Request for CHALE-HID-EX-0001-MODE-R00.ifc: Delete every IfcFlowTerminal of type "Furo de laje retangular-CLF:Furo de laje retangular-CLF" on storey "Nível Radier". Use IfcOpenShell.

First a look at what the model holds.

```python
import ifcopenshell
import ifcopenshell.util.element

model = ifcopenshell.open("CHALE-HID-EX-0001-MODE-R00.ifc")
print(model.schema)
storey = next(s for s in model.by_type("IfcBuildingStorey") if s.Name == "Nível Radier")
terminals = [e for e in ifcopenshell.util.element.get_decomposition(storey) if e.is_a("IfcFlowTerminal")]
seen = {}
for e in terminals:
    element_type = ifcopenshell.util.element.get_type(e)
    name = element_type.Name if element_type not in (None, e) else None
    seen[name] = seen.get(name, 0) + 1
for name, count in sorted(seen.items(), key=str):
    print(count, "x", name)
```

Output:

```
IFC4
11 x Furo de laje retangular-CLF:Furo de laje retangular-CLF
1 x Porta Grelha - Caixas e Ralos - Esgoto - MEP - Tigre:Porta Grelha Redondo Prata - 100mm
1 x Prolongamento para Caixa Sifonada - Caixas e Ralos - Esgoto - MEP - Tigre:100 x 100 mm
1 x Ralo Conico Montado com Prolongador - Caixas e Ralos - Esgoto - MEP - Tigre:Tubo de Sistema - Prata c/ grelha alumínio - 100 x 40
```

```python
import ifcopenshell
import ifcopenshell.api.root
import ifcopenshell.util.element

model = ifcopenshell.open("CHALE-HID-EX-0001-MODE-R00.ifc")

storey = next(s for s in model.by_type("IfcBuildingStorey") if s.Name == "Nível Radier")
terminals = [e for e in ifcopenshell.util.element.get_decomposition(storey) if e.is_a("IfcFlowTerminal")]
targets = [e for e in terminals if (t := ifcopenshell.util.element.get_type(e)) not in (None, e) and t.Name == "Furo de laje retangular-CLF:Furo de laje retangular-CLF"]

for e in targets:
    ifcopenshell.api.root.remove_product(model, product=e)
print(len(targets), "removed")

model.write("CHALE-HID-EX-0001-MODE-R00_edited.ifc")
```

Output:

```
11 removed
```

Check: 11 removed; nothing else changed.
